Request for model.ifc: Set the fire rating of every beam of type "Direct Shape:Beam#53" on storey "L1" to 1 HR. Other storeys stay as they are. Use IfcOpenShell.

First a look at what the model holds.

```python
import ifcopenshell
import ifcopenshell.util.element

model = ifcopenshell.open("model.ifc")
print(model.schema)
storey = next(s for s in model.by_type("IfcBuildingStorey") if s.Name == "L1")
beams = [e for e in ifcopenshell.util.element.get_decomposition(storey) if e.is_a("IfcBeam")]
seen = {}
for e in beams:
    element_type = ifcopenshell.util.element.get_type(e)
    key = (element_type.Name if element_type != e and element_type else None, ifcopenshell.util.element.get_pset(e, "Pset_BeamCommon", "FireRating"))
    seen[key] = seen.get(key, 0) + 1
for (name, value), count in sorted(seen.items(), key=str):
    print(count, "x", name, "|", value)
```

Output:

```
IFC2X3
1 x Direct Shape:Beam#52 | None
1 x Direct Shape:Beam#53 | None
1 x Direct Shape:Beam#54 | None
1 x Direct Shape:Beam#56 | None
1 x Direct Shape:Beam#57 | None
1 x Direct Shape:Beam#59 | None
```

```python
import ifcopenshell
import ifcopenshell.api.pset
import ifcopenshell.util.element

model = ifcopenshell.open("model.ifc")

storey = next(s for s in model.by_type("IfcBuildingStorey") if s.Name == "L1")
beams = [e for e in ifcopenshell.util.element.get_decomposition(storey) if e.is_a("IfcBeam")]

count = 0
for e in beams:
    element_type = ifcopenshell.util.element.get_type(e)
    if element_type in (None, e) or element_type.Name != "Direct Shape:Beam#53":
        continue
    # add_pset returns the element's existing set when there is one.
    pset = ifcopenshell.api.pset.add_pset(model, product=e, name="Pset_BeamCommon")
    ifcopenshell.api.pset.edit_pset(model, pset=pset, properties={"FireRating": "1 HR"})
    count += 1

print(count, "beams updated")

model.write("model_updated.ifc")
```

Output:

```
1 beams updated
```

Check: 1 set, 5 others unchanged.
